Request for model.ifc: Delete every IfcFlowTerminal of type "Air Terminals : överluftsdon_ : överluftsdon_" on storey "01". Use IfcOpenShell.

First a look at what the model holds.

```python
import ifcopenshell
import ifcopenshell.util.element

model = ifcopenshell.open("model.ifc")
print(model.schema)
storey = next(s for s in model.by_type("IfcBuildingStorey") if s.Name == "01")
terminals = [e for e in ifcopenshell.util.element.get_decomposition(storey) if e.is_a("IfcFlowTerminal")]
seen = {}
for e in terminals:
    element_type = ifcopenshell.util.element.get_type(e)
    name = element_type.Name if element_type not in (None, e) else None
    seen[name] = seen.get(name, 0) + 1
for name, count in sorted(seen.items(), key=str):
    print(count, "x", name)
```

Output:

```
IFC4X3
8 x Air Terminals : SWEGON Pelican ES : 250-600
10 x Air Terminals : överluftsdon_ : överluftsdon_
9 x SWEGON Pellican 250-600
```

```python
import ifcopenshell
import ifcopenshell.api.root
import ifcopenshell.util.element

model = ifcopenshell.open("model.ifc")

storey = next(s for s in model.by_type("IfcBuildingStorey") if s.Name == "01")
terminals = [e for e in ifcopenshell.util.element.get_decomposition(storey) if e.is_a("IfcFlowTerminal")]
targets = [e for e in terminals if (t := ifcopenshell.util.element.get_type(e)) not in (None, e) and t.Name == "Air Terminals : överluftsdon_ : överluftsdon_"]

for e in targets:
    ifcopenshell.api.root.remove_product(model, product=e)
print(len(targets), "removed")

model.write("model-out.ifc")
```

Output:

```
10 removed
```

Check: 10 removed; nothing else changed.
